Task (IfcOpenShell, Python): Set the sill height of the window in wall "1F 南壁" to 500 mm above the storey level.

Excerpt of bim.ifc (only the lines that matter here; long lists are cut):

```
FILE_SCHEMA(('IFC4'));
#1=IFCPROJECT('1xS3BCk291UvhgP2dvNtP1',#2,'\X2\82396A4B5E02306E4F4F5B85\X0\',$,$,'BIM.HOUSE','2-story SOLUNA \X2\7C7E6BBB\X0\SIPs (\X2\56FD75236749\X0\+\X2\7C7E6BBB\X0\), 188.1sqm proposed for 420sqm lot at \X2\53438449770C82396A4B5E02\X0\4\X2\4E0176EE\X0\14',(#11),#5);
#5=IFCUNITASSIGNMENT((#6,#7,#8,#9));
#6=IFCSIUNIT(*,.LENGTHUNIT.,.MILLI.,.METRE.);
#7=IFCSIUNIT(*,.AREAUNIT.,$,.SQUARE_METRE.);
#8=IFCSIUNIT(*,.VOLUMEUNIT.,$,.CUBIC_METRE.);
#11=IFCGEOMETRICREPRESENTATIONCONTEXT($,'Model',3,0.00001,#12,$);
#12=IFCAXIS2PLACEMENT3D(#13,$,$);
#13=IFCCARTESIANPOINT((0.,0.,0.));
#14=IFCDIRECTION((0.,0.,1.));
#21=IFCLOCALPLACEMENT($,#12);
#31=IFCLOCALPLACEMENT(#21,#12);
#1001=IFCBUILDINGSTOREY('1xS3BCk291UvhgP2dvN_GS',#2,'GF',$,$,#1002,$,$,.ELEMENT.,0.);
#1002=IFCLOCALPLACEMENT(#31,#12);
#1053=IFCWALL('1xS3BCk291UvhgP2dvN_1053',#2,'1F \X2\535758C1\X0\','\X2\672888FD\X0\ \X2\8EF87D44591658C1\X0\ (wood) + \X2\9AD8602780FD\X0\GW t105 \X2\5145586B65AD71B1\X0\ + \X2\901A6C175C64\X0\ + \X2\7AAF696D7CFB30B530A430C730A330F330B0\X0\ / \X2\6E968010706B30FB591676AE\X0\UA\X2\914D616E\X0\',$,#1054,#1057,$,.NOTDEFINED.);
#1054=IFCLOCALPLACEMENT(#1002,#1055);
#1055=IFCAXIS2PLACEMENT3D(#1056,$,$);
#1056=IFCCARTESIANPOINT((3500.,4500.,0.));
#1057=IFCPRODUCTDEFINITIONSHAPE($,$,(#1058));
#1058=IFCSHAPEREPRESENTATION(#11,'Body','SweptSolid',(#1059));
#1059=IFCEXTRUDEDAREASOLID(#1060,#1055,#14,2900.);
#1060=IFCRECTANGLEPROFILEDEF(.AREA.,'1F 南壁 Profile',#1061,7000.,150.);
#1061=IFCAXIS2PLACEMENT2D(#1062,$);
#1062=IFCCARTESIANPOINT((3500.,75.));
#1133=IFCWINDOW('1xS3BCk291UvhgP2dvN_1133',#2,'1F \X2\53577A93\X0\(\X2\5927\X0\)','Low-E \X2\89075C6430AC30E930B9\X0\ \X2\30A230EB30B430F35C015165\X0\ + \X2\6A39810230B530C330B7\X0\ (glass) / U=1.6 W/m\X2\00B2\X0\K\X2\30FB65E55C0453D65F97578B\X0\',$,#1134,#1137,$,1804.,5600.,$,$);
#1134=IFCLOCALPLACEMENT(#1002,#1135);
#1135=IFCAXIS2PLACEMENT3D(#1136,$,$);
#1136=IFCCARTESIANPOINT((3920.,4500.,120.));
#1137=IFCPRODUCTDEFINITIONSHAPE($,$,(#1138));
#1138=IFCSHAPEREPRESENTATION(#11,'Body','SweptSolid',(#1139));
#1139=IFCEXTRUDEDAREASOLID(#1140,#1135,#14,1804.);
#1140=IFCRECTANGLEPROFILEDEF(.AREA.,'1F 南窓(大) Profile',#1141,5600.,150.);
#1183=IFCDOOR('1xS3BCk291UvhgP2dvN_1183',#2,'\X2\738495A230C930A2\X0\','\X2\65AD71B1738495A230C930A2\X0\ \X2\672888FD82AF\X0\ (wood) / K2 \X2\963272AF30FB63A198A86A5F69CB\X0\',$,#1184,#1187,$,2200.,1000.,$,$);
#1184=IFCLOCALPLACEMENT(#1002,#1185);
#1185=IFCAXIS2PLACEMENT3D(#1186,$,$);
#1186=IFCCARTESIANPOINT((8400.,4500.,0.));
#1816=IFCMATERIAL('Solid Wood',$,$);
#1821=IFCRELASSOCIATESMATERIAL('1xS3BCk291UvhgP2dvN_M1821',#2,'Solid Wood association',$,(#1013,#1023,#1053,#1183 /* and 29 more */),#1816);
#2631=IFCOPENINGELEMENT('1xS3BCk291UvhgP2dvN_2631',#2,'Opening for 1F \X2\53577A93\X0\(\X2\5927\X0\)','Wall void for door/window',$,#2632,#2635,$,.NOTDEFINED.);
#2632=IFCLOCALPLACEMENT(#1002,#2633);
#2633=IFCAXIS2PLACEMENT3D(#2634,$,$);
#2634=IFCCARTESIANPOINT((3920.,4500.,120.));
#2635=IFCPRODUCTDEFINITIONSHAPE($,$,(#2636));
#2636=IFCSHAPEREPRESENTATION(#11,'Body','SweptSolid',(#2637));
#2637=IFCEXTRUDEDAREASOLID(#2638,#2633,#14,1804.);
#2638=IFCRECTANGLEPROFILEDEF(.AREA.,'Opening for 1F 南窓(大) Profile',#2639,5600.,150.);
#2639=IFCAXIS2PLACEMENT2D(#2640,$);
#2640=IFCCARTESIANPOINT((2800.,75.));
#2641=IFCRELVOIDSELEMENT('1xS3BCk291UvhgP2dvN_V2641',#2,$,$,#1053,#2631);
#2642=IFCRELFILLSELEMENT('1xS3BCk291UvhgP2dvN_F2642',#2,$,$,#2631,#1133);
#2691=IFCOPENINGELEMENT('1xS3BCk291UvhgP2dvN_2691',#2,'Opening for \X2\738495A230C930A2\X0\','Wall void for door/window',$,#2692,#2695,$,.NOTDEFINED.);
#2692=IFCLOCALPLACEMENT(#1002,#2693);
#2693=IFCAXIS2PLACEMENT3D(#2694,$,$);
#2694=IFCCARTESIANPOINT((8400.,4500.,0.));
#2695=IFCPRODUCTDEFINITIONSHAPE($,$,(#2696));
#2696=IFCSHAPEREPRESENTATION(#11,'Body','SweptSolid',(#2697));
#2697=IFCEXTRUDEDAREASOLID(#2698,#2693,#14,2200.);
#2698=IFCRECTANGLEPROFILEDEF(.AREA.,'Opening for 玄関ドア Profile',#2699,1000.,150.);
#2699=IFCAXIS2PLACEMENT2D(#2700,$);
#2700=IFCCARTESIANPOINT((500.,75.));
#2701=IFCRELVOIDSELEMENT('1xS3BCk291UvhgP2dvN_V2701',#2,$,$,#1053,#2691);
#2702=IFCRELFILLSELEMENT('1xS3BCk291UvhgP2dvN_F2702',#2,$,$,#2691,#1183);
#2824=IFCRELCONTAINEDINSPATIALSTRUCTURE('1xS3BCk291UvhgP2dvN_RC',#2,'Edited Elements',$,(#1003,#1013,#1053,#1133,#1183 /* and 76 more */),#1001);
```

```python
import numpy as np
import ifcopenshell
import ifcopenshell.api.geometry
import ifcopenshell.geom
import ifcopenshell.util.element
import ifcopenshell.util.placement
import ifcopenshell.util.shape
import ifcopenshell.util.unit

model = ifcopenshell.open("bim.ifc")
unit_scale = ifcopenshell.util.unit.calculate_unit_scale(model)

window = model.by_id(1133)
opening = window.FillsVoids[0].RelatingOpeningElement
storey = ifcopenshell.util.element.get_container(window, ifc_class="IfcBuildingStorey")
level = ifcopenshell.util.placement.get_local_placement(storey.ObjectPlacement)[2, 3]

# The opening's origin need not be at the sill, so measure its lowest point.
shape = ifcopenshell.geom.create_shape(ifcopenshell.geom.settings(), opening)
bottom = ifcopenshell.util.shape.get_shape_bottom_elevation(shape, shape.geometry) / unit_scale
dz = level + 500.0 - bottom

shift = np.array([0.0, 0.0, dz])
# The window is not placed relative to its opening, so move both.
for product in (opening, window):
    matrix = ifcopenshell.util.placement.get_local_placement(product.ObjectPlacement)
    matrix[:3, 3] += shift
    ifcopenshell.api.geometry.edit_object_placement(model, product=product, matrix=matrix, is_si=False)

print(f"moved by {dz * unit_scale:+.3f} m")

model.write("bim_rev.ifc")
```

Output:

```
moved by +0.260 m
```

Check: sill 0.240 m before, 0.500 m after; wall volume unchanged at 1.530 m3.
